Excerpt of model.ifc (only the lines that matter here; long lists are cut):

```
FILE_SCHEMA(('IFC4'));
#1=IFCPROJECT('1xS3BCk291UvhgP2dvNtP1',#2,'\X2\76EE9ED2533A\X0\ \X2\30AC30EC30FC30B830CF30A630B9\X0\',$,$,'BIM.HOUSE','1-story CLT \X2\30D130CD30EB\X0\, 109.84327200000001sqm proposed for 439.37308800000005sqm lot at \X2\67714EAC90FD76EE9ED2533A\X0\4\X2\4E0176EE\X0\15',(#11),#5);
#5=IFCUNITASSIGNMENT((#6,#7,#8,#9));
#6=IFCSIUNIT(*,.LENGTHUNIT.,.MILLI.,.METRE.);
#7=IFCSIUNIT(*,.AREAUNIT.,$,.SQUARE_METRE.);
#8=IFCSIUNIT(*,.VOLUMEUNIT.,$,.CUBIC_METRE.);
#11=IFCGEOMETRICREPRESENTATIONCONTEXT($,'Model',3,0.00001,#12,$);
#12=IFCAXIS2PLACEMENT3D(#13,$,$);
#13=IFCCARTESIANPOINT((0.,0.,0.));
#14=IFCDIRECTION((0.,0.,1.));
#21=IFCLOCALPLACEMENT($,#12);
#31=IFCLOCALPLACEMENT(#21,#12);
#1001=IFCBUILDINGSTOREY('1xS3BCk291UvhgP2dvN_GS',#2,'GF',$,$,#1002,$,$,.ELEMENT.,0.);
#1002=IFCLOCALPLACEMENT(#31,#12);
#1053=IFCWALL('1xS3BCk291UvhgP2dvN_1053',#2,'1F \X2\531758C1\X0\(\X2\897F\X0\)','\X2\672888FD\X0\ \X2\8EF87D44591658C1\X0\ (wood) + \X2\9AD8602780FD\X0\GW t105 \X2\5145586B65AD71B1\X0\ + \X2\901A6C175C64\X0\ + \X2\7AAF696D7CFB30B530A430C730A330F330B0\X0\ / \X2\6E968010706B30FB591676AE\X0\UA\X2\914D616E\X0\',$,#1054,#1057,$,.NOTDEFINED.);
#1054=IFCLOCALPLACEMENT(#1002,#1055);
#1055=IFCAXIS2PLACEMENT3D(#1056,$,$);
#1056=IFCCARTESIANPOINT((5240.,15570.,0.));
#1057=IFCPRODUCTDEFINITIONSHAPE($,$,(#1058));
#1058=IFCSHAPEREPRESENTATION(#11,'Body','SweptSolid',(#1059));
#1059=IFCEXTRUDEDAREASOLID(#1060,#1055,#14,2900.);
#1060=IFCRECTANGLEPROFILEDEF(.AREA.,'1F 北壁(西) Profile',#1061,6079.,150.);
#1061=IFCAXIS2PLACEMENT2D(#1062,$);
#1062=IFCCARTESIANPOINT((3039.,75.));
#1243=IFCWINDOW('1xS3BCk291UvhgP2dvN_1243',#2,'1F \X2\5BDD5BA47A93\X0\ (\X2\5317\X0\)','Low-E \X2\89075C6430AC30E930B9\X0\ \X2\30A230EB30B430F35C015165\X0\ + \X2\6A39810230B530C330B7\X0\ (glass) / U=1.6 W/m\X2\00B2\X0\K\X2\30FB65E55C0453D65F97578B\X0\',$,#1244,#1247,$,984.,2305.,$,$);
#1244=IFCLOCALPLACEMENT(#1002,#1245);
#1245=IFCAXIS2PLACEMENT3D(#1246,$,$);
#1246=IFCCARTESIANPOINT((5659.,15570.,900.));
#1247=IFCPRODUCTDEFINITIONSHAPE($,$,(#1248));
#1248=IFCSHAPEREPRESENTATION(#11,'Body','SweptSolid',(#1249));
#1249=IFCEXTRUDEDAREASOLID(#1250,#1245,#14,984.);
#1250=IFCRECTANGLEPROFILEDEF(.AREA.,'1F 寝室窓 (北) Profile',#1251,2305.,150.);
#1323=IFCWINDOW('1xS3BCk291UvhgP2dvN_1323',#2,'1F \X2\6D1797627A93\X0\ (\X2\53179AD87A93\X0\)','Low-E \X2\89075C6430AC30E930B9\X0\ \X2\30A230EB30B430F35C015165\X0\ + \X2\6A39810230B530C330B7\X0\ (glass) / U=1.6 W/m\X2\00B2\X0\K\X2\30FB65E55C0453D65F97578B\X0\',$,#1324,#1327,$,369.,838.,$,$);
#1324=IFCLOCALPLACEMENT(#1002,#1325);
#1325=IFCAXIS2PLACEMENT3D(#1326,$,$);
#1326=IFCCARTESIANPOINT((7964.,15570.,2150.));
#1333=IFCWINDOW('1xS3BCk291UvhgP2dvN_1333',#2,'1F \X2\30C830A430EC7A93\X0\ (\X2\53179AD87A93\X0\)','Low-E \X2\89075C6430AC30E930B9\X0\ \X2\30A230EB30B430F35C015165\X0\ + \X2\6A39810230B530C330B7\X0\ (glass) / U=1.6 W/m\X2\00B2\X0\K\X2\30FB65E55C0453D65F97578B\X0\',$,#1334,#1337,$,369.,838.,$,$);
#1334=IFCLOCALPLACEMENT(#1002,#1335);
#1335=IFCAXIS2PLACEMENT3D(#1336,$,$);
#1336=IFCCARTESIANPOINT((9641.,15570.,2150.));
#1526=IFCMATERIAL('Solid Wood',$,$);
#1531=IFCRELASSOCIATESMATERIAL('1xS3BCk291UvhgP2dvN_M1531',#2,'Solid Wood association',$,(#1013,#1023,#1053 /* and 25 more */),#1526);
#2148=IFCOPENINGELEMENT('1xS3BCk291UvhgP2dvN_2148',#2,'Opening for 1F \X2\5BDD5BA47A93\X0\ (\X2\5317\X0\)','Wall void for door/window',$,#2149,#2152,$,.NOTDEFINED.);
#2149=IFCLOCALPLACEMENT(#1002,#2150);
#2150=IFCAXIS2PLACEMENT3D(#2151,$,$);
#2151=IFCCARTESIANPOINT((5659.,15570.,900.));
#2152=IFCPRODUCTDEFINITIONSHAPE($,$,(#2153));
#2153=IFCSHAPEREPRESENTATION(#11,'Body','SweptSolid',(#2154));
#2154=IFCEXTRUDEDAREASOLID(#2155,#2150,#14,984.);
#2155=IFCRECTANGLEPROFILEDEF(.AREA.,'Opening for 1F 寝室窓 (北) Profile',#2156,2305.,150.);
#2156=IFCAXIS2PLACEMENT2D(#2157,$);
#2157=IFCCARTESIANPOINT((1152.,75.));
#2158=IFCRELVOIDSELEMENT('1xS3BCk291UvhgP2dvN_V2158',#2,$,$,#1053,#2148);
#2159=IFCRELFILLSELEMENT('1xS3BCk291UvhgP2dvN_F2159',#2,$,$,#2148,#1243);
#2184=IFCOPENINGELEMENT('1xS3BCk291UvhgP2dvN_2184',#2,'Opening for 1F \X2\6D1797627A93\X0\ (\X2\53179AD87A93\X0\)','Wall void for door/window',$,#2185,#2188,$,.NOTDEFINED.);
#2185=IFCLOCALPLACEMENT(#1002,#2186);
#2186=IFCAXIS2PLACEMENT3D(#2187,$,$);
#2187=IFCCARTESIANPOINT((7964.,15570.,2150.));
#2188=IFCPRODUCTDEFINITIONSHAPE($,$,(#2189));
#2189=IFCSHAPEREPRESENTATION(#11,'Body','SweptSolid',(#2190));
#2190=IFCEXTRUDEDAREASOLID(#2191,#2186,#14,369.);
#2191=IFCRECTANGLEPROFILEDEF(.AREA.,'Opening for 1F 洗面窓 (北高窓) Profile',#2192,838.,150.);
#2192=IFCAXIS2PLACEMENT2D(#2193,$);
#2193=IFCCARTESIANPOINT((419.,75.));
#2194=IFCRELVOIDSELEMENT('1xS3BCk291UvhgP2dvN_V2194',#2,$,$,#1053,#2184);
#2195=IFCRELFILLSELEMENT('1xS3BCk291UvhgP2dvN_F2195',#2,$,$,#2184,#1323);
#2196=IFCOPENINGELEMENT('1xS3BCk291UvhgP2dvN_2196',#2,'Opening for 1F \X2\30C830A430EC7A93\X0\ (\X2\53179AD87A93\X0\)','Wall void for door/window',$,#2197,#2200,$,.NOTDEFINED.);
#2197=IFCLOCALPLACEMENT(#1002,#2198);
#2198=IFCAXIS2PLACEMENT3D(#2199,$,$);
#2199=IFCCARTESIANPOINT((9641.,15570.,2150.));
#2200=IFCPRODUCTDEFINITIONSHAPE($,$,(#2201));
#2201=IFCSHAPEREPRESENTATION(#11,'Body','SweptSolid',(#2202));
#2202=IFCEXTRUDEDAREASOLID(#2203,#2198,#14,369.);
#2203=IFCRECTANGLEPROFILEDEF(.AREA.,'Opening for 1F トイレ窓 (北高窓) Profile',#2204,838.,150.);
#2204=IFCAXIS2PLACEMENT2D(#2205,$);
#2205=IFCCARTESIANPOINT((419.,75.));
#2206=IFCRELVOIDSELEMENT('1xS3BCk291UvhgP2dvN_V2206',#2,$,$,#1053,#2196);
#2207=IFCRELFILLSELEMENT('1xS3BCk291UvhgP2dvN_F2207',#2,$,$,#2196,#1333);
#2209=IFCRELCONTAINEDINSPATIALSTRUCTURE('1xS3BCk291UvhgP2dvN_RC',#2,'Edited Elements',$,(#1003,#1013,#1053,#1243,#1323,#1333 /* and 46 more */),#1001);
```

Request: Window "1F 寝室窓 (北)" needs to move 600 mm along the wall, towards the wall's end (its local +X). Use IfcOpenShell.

```python
import ifcopenshell
import ifcopenshell.api.geometry
import ifcopenshell.util.placement
import ifcopenshell.util.unit

model = ifcopenshell.open("model.ifc")
unit_scale = ifcopenshell.util.unit.calculate_unit_scale(model)

window = model.by_guid("1xS3BCk291UvhgP2dvN_1243")
opening = window.FillsVoids[0].RelatingOpeningElement
wall = opening.VoidsElements[0].RelatingBuildingElement

wall_matrix = ifcopenshell.util.placement.get_local_placement(wall.ObjectPlacement)
shift = wall_matrix[:3, 0] * 0.6 / unit_scale
before = ifcopenshell.util.placement.get_local_placement(window.ObjectPlacement)[:3, 3].copy()

# The window is not placed relative to its opening, so move both.
for product in (opening, window):
    matrix = ifcopenshell.util.placement.get_local_placement(product.ObjectPlacement)
    matrix[:3, 3] += shift
    ifcopenshell.api.geometry.edit_object_placement(model, product=product, matrix=matrix, is_si=False)

after = ifcopenshell.util.placement.get_local_placement(window.ObjectPlacement)[:3, 3]
print("window moved by", (after - before).round(3) + 0.0)

model.write("model-out.ifc")
```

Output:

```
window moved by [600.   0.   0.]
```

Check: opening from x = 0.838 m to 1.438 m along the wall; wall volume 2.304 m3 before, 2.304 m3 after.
